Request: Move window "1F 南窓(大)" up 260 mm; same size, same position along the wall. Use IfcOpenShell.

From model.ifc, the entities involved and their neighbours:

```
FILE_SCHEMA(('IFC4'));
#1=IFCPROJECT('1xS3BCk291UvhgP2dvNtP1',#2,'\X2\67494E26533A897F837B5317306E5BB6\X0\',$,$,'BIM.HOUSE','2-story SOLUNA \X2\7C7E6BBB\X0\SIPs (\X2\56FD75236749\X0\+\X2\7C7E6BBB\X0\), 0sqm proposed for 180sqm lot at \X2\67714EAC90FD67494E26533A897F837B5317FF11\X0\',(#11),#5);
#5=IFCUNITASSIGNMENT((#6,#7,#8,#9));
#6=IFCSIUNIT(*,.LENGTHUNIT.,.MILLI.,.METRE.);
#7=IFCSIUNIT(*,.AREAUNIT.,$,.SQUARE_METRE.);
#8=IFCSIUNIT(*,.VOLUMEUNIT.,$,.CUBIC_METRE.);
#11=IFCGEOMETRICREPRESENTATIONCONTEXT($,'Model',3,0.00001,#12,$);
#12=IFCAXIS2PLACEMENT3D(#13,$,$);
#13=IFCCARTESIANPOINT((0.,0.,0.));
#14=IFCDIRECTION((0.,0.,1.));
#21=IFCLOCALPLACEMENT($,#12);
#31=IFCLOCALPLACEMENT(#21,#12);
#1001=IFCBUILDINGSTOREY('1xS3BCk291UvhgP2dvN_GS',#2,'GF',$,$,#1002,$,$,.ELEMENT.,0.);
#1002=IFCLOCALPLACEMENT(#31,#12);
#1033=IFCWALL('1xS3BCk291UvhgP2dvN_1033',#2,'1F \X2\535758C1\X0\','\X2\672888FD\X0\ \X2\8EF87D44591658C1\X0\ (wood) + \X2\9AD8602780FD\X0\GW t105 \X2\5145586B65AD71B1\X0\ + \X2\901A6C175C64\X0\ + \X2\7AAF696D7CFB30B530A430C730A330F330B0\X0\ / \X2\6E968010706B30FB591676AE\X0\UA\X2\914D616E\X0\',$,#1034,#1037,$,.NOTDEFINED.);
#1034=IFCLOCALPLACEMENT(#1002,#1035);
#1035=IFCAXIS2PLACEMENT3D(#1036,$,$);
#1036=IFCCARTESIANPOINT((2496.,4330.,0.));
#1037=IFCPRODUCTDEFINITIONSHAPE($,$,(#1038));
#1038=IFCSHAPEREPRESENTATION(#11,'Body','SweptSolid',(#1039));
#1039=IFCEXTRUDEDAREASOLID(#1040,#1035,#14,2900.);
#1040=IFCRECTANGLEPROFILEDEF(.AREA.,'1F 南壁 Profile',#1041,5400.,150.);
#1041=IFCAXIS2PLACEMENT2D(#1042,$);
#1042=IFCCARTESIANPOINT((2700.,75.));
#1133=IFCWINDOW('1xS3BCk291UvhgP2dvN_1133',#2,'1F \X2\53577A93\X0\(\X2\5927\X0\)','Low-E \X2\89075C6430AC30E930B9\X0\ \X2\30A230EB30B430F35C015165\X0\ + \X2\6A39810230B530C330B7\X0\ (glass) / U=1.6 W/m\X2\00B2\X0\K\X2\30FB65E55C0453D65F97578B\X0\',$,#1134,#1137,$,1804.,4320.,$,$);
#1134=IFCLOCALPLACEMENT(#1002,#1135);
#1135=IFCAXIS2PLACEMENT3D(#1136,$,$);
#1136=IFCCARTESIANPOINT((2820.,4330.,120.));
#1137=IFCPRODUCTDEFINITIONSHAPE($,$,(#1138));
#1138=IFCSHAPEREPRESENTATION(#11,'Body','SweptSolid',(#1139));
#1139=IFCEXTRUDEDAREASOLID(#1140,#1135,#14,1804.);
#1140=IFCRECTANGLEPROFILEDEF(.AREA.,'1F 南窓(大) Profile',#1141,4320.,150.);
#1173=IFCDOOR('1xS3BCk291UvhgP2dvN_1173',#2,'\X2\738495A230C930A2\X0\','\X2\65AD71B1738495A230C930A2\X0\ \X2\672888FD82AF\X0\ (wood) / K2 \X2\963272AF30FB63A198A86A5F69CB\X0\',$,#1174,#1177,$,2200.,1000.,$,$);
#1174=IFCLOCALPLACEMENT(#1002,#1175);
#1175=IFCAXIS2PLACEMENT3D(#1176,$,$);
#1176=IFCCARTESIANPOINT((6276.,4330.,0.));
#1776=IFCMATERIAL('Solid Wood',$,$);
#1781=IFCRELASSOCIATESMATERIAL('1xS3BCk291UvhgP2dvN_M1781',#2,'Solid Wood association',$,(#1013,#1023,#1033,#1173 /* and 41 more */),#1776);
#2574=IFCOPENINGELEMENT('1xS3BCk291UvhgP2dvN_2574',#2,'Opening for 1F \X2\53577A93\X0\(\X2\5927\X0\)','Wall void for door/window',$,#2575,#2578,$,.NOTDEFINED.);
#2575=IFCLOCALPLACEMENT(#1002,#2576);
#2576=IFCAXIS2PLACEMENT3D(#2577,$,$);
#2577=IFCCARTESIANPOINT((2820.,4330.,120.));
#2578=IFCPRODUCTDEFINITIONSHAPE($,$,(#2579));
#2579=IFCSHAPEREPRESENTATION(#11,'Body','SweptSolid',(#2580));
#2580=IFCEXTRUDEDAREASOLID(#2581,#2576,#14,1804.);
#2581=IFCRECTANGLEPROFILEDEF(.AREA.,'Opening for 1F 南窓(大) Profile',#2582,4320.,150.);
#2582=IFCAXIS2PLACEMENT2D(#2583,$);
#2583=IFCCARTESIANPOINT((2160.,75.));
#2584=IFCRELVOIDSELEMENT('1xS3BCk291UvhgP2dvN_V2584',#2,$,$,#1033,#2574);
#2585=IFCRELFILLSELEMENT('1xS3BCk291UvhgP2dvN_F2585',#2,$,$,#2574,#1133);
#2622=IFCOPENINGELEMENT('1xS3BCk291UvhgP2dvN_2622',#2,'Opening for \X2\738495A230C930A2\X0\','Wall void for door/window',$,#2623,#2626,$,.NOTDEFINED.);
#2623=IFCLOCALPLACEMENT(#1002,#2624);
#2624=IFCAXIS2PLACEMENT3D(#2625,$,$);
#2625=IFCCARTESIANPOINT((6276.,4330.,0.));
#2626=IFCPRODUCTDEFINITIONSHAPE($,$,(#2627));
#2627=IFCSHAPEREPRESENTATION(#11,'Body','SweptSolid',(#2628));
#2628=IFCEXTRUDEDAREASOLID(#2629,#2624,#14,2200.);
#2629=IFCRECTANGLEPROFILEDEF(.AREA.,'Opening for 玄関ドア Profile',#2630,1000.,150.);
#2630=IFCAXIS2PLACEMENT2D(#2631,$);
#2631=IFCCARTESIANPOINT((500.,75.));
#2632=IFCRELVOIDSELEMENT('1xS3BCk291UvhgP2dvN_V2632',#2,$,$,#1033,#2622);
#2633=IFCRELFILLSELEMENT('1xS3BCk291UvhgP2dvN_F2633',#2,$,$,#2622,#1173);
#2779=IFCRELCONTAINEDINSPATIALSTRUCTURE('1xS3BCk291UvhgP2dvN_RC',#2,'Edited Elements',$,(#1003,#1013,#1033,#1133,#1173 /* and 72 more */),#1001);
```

```python
import numpy as np
import ifcopenshell
import ifcopenshell.api.geometry
import ifcopenshell.util.placement
import ifcopenshell.util.unit

model = ifcopenshell.open("model.ifc")
unit_scale = ifcopenshell.util.unit.calculate_unit_scale(model)

window = model.by_id(1133)
opening = window.FillsVoids[0].RelatingOpeningElement
dz = 0.26 / unit_scale

shift = np.array([0.0, 0.0, dz])
# The window is not placed relative to its opening, so move both.
for product in (opening, window):
    matrix = ifcopenshell.util.placement.get_local_placement(product.ObjectPlacement)
    matrix[:3, 3] += shift
    ifcopenshell.api.geometry.edit_object_placement(model, product=product, matrix=matrix, is_si=False)

print(f"moved by {dz * unit_scale:+.3f} m")

model.write("model_edited.ifc")
```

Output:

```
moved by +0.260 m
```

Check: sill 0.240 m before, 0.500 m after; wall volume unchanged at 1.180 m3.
